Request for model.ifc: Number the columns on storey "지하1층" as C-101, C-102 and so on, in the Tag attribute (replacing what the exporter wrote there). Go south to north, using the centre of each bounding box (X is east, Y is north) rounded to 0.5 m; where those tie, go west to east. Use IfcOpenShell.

First a look at what the model holds.

```python
import ifcopenshell
import ifcopenshell.util.element
import ifcopenshell.util.placement

model = ifcopenshell.open("model.ifc")
print(model.schema)
storey = next(s for s in model.by_type("IfcBuildingStorey") if s.Name == "지하1층")
columns = [e for e in ifcopenshell.util.element.get_decomposition(storey) if e.is_a("IfcColumn")]
for e in sorted(columns, key=lambda e: e.id()):
    origin = ifcopenshell.util.placement.get_local_placement(e.ObjectPlacement)[:3, 3]
    print(e.id(), e.Tag, e.Name, origin.round(2) + 0.0, sep=" | ")
```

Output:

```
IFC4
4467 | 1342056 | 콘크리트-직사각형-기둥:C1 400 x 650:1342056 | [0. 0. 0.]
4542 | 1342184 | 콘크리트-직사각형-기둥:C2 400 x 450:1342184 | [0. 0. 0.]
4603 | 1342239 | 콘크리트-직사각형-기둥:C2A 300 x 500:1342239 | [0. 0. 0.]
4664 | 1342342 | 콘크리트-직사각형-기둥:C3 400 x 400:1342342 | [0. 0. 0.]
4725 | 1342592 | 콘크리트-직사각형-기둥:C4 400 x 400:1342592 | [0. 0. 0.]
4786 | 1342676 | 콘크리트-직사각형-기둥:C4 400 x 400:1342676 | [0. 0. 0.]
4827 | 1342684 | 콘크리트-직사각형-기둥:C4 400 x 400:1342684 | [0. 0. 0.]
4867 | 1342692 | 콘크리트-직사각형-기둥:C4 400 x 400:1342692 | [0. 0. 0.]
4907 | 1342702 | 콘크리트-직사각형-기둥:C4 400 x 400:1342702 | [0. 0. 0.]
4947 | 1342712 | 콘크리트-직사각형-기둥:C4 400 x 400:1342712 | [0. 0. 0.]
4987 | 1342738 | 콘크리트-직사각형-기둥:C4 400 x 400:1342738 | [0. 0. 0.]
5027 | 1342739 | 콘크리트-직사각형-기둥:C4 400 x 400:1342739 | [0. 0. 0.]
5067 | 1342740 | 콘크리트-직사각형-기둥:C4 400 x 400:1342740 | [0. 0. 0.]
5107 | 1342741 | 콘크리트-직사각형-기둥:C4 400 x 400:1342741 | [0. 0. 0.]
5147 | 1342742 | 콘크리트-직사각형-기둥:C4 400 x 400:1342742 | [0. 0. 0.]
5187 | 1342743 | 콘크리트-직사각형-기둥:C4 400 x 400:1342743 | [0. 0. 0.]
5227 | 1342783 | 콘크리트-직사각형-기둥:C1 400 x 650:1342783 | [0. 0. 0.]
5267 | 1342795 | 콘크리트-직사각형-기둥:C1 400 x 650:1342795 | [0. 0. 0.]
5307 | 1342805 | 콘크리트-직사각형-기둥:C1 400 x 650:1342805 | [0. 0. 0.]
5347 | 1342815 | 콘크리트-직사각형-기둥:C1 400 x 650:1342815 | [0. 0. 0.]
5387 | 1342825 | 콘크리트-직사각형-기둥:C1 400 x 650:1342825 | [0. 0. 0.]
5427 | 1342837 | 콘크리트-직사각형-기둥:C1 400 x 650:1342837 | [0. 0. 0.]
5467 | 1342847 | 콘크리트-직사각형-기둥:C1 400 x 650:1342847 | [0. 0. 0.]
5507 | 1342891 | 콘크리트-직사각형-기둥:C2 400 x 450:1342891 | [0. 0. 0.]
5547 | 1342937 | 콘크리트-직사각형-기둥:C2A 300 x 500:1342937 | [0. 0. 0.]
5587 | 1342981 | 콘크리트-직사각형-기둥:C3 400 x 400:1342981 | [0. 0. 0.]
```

```python
import ifcopenshell
import ifcopenshell.geom
import ifcopenshell.util.element
import ifcopenshell.util.shape

model = ifcopenshell.open("model.ifc")
settings = ifcopenshell.geom.settings()
settings.set("use-world-coords", True)


def centre(element):
    shape = ifcopenshell.geom.create_shape(settings, element)
    return ifcopenshell.util.shape.get_bbox_centroid(shape.geometry)


storey = next(s for s in model.by_type("IfcBuildingStorey") if s.Name == "지하1층")
columns = [e for e in ifcopenshell.util.element.get_decomposition(storey) if e.is_a("IfcColumn")]

# Insertion points can sit at a corner or the storey origin, so sort by the geometry (in metres).
centres = {e: centre(e) for e in columns}
columns.sort(key=lambda e: (round(centres[e][1] / 0.5), centres[e][0]))

for i, e in enumerate(columns, start=1):
    number = f"C-1{i:02d}"
    e.Tag = number
    print(e.id(), number)

model.write("model_edited.ifc")
```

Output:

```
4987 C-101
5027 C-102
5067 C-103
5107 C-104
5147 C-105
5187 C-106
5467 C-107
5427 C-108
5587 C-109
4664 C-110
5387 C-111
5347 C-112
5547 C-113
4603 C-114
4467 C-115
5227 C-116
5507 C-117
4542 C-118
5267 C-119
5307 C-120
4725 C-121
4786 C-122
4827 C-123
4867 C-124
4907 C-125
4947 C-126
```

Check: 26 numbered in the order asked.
